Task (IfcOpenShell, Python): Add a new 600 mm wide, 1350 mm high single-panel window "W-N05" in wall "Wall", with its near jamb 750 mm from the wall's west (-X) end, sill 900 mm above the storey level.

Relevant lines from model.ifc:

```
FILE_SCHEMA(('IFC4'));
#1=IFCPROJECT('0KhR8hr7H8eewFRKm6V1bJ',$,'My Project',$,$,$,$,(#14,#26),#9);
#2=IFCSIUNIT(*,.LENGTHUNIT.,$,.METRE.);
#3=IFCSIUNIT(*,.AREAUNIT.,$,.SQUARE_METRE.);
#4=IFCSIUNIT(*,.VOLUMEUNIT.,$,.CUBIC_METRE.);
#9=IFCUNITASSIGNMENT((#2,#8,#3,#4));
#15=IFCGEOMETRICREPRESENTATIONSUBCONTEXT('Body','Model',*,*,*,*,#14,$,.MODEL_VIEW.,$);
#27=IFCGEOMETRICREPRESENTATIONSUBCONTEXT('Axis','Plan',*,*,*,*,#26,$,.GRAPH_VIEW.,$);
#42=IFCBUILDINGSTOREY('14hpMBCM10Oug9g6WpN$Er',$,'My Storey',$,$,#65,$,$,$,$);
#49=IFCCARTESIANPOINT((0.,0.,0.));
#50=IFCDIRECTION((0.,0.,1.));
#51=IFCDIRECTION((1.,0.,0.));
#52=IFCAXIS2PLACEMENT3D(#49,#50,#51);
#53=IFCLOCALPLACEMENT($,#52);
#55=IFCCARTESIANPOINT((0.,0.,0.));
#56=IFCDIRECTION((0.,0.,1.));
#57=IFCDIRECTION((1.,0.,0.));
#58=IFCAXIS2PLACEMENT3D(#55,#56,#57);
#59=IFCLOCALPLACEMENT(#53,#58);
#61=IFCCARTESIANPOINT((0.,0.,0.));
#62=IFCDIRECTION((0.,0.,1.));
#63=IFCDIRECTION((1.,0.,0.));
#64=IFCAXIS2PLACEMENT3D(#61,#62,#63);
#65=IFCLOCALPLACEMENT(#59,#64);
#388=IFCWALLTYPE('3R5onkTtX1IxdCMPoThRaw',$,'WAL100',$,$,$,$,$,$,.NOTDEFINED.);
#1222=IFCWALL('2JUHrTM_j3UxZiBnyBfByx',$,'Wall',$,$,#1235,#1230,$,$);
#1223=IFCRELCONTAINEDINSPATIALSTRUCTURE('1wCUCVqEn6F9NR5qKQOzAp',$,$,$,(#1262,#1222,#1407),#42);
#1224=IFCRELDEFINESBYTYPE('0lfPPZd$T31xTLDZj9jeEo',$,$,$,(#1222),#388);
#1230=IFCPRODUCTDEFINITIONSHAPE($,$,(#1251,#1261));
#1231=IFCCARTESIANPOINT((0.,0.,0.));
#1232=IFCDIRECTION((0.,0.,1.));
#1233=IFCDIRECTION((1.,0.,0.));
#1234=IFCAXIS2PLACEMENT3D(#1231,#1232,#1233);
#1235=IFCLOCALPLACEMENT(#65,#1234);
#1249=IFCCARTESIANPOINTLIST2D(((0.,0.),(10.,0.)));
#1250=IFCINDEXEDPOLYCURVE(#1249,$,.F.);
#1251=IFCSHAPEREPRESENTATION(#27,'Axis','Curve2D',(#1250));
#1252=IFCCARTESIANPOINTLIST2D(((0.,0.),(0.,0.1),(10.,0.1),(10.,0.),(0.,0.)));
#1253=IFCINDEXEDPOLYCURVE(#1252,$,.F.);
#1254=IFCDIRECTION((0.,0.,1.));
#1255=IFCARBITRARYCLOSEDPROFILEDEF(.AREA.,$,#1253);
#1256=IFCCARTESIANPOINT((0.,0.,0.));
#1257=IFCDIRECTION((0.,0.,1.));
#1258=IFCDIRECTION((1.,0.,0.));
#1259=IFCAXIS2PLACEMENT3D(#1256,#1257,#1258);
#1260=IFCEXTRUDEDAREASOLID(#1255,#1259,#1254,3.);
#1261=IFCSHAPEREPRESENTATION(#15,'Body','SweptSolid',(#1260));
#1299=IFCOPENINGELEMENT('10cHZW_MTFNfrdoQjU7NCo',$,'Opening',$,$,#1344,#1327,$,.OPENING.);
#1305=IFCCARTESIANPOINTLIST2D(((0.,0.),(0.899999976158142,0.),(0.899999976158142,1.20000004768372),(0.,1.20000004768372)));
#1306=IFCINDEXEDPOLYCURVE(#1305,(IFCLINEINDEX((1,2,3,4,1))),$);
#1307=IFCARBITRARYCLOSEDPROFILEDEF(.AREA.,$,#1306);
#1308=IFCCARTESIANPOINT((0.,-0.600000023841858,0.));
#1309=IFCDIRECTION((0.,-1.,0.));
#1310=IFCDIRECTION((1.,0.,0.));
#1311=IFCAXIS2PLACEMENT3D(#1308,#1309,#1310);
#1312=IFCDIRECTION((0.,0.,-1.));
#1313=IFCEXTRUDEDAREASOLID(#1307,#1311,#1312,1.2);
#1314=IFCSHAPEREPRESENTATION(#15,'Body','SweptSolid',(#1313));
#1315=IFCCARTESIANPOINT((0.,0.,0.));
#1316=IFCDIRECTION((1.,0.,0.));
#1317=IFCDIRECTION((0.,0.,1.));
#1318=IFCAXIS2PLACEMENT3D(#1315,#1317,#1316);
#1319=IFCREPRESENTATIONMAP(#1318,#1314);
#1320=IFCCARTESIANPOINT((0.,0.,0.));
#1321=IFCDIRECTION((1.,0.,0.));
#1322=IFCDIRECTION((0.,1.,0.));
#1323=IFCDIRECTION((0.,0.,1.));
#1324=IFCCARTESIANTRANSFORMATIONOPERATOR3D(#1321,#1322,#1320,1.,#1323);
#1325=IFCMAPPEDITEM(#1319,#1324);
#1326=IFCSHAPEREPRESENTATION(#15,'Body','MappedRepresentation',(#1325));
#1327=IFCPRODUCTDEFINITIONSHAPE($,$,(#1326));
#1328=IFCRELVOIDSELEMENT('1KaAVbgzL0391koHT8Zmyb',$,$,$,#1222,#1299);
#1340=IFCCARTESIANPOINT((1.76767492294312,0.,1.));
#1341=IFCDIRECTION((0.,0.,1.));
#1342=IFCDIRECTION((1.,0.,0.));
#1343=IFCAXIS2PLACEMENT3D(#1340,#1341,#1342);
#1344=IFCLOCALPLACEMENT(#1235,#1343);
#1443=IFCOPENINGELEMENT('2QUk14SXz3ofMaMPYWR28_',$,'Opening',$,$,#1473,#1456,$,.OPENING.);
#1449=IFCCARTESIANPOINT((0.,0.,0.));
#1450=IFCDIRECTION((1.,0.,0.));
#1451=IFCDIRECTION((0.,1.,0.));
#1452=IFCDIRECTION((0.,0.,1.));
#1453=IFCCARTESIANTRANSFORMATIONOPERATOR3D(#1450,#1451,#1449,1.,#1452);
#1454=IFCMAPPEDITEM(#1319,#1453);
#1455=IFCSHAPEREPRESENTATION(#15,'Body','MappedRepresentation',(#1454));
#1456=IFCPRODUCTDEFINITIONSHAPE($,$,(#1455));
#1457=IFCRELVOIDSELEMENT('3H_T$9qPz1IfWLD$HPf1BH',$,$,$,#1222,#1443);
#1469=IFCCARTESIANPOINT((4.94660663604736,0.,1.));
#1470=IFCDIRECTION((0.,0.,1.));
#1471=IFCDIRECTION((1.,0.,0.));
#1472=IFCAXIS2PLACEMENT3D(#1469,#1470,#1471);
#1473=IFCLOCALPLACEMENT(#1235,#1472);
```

```python
import numpy as np
import ifcopenshell
import ifcopenshell.api.feature
import ifcopenshell.api.geometry
import ifcopenshell.api.root
import ifcopenshell.api.spatial
import ifcopenshell.geom
import ifcopenshell.util.element
import ifcopenshell.util.placement
import ifcopenshell.util.representation
import ifcopenshell.util.shape
import ifcopenshell.util.unit

model = ifcopenshell.open("model.ifc")
unit_scale = ifcopenshell.util.unit.calculate_unit_scale(model)
settings = ifcopenshell.geom.settings()


def volume(element):
    """Net volume in cubic metres, openings subtracted."""
    shape = ifcopenshell.geom.create_shape(settings, element)
    return ifcopenshell.util.shape.get_volume(shape.geometry)


wall = model.by_guid("2JUHrTM_j3UxZiBnyBfByx")
storey = ifcopenshell.util.element.get_container(wall, ifc_class="IfcBuildingStorey")
context = ifcopenshell.util.representation.get_context(model, "Model", "Body", "MODEL_VIEW")
before = volume(wall)

width, height, from_end, sill = 0.6, 1.35, 0.75, 0.9  # metres

# The wall runs along its own X axis, and the end named is its -X end.
wall_shape = ifcopenshell.geom.create_shape(settings, wall)
x, y, z = ifcopenshell.util.shape.get_vertices(wall_shape.geometry).T
start = x.min() + from_end
face, thickness = float(y.min()), float(y.max() - y.min())
wall_matrix = ifcopenshell.util.placement.get_local_placement(wall.ObjectPlacement)
level = ifcopenshell.util.placement.get_local_placement(storey.ObjectPlacement)[2, 3]


def in_wall(x, y):
    """Placement at x, y metres in the wall's axes, at sill height."""
    matrix = wall_matrix.copy()
    matrix[:, 3] = wall_matrix @ np.array([x / unit_scale, y / unit_scale, 0.0, 1.0])
    matrix[2, 3] = level + sill / unit_scale
    return matrix


# Opening: a box that overshoots both wall faces by 50 mm.
opening = ifcopenshell.api.root.create_entity(model, ifc_class="IfcOpeningElement", predefined_type="OPENING")
box = ifcopenshell.api.geometry.add_wall_representation(
    model, context=context, length=width, height=height, thickness=thickness + 0.1
)
ifcopenshell.api.geometry.assign_representation(model, product=opening, representation=box)
ifcopenshell.api.geometry.edit_object_placement(model, product=opening, matrix=in_wall(start, face - 0.05), is_si=False)
ifcopenshell.api.feature.add_feature(model, feature=opening, element=wall)

window = ifcopenshell.api.root.create_entity(model, ifc_class="IfcWindow", name="W-N05", predefined_type="WINDOW")
window.OverallWidth, window.OverallHeight = width / unit_scale, height / unit_scale
window.PartitioningType = "SINGLE_PANEL"
body = ifcopenshell.api.geometry.add_window_representation(
    model,
    context=context,
    overall_width=window.OverallWidth,
    overall_height=window.OverallHeight,
    partition_type="SINGLE_PANEL",
)
ifcopenshell.api.geometry.assign_representation(model, product=window, representation=body)
ifcopenshell.api.spatial.assign_container(model, products=[window], relating_structure=storey)
ifcopenshell.api.feature.add_filling(model, opening=opening, element=window)

# Centre the window in the wall's thickness.
ifcopenshell.api.geometry.edit_object_placement(model, product=window, matrix=in_wall(start, face), is_si=False)
window_shape = ifcopenshell.geom.create_shape(settings, window)
depth = ifcopenshell.util.shape.get_vertices(window_shape.geometry)[:, 1]
offset = face + thickness / 2 - (depth.min() + depth.max()) / 2
ifcopenshell.api.geometry.edit_object_placement(model, product=window, matrix=in_wall(start, offset), is_si=False)

after = volume(wall)

print(f"wall volume {before:.3f} -> {after:.3f} m3")

model.write("model_updated.ifc")
```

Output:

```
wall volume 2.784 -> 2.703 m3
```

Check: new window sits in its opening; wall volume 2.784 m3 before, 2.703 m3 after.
